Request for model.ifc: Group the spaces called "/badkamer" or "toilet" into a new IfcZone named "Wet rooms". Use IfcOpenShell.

First a look at what the model holds.

```python
import ifcopenshell

model = ifcopenshell.open("model.ifc")
print(model.schema)
seen = {}
for space in model.by_type("IfcSpace"):
    seen[space.Name] = seen.get(space.Name, 0) + 1
for name, count in sorted(seen.items(), key=str):
    print(count, "x", name)
print("zones:", [z.Name for z in model.by_type("IfcZone")][:20])
```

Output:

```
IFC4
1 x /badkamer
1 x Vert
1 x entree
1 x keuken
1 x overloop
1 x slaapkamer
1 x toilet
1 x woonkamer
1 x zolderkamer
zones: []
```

```python
import ifcopenshell
import ifcopenshell.api.group
import ifcopenshell.api.root

model = ifcopenshell.open("model.ifc")

names = {"/badkamer", "toilet"}
spaces = [s for s in model.by_type("IfcSpace") if s.Name in names]

zone = ifcopenshell.api.root.create_entity(model, ifc_class="IfcZone", name="Wet rooms")
ifcopenshell.api.group.assign_group(model, products=spaces, group=zone)
print(len(spaces), "spaces in", zone.Name)

model.write("model_updated.ifc")
```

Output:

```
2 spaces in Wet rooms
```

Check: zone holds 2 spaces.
